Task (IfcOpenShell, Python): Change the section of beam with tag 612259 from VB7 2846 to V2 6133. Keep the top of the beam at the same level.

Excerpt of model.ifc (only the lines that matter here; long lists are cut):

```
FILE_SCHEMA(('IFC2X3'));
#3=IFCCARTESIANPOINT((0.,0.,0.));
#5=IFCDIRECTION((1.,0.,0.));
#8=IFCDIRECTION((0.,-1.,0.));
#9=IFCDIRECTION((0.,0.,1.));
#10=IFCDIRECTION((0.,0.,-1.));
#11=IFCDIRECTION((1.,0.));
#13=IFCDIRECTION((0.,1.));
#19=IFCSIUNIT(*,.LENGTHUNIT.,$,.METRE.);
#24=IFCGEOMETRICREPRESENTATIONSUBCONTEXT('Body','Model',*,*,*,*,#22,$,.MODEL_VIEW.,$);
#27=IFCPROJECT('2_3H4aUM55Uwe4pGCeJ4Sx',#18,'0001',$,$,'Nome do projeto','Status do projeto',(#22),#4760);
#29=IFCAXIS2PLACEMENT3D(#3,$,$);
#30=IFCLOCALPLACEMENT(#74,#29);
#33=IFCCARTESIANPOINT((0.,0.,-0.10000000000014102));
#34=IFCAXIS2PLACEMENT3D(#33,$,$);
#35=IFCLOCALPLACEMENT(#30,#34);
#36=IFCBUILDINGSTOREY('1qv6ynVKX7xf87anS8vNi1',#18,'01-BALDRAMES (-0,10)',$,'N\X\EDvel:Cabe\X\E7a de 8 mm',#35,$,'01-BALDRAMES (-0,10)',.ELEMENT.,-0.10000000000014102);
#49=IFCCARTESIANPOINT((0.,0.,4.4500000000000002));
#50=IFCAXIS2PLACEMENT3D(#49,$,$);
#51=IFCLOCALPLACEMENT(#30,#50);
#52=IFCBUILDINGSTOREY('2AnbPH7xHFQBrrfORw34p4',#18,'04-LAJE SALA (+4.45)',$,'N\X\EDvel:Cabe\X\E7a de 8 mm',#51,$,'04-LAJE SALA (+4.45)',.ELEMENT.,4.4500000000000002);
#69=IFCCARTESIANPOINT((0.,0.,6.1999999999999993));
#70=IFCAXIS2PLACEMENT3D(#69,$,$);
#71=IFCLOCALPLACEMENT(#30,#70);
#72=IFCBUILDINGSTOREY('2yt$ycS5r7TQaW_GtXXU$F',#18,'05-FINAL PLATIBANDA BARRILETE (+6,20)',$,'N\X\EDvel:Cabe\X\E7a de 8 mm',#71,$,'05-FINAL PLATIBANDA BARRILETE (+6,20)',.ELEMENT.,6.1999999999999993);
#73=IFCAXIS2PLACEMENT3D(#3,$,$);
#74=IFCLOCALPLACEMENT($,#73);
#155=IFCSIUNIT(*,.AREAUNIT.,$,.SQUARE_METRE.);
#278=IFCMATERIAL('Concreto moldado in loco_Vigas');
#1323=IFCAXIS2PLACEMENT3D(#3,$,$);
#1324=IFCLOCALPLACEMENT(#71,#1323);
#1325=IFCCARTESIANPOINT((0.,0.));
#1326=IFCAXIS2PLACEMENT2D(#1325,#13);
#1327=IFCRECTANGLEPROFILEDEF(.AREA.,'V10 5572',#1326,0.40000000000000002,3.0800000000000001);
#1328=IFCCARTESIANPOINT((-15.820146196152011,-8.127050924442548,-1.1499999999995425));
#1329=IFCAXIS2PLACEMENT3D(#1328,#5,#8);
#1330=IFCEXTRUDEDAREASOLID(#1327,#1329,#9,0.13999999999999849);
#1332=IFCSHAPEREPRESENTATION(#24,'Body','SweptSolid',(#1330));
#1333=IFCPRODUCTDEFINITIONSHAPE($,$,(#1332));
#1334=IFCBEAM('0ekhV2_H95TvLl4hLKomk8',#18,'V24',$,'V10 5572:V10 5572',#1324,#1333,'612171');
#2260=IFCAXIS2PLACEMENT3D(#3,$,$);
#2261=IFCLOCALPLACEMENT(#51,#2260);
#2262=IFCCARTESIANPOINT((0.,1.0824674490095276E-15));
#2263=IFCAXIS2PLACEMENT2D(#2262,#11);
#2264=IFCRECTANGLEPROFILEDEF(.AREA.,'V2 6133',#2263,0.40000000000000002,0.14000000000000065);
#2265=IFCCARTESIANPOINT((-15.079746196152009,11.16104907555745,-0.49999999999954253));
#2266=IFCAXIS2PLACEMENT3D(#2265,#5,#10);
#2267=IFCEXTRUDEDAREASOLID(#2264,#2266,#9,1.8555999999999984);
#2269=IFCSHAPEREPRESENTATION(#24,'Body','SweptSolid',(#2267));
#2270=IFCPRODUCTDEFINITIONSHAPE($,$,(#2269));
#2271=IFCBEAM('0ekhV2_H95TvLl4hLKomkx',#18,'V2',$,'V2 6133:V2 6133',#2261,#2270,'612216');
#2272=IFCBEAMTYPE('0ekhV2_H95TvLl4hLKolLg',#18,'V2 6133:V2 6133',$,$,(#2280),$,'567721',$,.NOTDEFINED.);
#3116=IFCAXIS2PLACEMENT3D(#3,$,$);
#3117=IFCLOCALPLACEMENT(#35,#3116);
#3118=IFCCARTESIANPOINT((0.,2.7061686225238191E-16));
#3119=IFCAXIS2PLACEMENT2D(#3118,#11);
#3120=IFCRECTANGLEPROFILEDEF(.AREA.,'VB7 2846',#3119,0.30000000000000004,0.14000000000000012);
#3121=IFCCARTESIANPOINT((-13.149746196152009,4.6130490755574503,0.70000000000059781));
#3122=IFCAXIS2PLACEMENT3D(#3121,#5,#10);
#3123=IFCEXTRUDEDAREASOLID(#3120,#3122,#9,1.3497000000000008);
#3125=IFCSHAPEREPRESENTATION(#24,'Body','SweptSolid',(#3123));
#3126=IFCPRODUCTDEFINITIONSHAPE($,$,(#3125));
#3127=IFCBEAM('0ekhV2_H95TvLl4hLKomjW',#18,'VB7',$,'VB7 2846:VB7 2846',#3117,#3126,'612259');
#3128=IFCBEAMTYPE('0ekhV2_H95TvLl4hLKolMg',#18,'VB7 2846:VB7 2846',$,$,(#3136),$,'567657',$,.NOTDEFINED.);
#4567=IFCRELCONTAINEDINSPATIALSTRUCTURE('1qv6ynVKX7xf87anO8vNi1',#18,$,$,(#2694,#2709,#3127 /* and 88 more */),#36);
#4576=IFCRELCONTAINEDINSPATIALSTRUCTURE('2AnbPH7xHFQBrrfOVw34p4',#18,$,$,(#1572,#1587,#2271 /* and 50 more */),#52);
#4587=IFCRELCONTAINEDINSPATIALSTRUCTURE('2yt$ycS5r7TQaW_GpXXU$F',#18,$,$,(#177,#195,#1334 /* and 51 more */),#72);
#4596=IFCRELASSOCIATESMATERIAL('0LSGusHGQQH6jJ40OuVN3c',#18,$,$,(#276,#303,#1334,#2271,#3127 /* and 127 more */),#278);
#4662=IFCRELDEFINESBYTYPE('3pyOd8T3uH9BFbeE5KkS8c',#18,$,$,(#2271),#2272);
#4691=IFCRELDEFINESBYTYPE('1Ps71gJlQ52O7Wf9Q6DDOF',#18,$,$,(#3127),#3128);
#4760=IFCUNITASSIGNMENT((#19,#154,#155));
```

```python
import ifcopenshell
import ifcopenshell.api.type
import ifcopenshell.util.element
import ifcopenshell.util.representation

model = ifcopenshell.open("model.ifc")

member = model.by_guid("0ekhV2_H95TvLl4hLKomjW")
source = next(p for p in model.by_type("IfcRectangleProfileDef") if p.ProfileName == "V2 6133")

body = ifcopenshell.util.representation.get_representation(member, "Model", "Body")
solid = body.Items[0]
old_profile = solid.SweptArea

# Copy the section's sizes but keep this member's own profile position.
profile = ifcopenshell.util.element.copy(model, source)
# Profiles are centred, so shift by half the change in depth to hold the top.
shift = (old_profile.XDim - profile.XDim) / 2
x, y = old_profile.Position.Location.Coordinates
up = (-1.0, 0.0)  # upwards, in the solid's own plane
location = model.createIfcCartesianPoint((x + up[0] * shift, y + up[1] * shift))
profile.Position = model.createIfcAxis2Placement2D(location, old_profile.Position.RefDirection)
solid.SweptArea = profile
if not model.get_total_inverses(old_profile):
    ifcopenshell.util.element.remove_deep2(model, old_profile)

new_type = model.by_guid("0ekhV2_H95TvLl4hLKolLg")
ifcopenshell.api.type.assign_type(
    model, related_objects=[member], relating_type=new_type, should_map_representations=False
)
member.ObjectType = "V2 6133:V2 6133"

print(solid.SweptArea)

model.write("model-out.ifc")
```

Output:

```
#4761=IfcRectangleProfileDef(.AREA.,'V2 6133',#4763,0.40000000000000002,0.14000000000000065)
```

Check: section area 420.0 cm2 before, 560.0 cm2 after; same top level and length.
